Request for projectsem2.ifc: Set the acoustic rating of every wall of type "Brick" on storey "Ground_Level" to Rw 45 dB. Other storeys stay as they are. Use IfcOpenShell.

First a look at what the model holds.

```python
import ifcopenshell
import ifcopenshell.util.element

model = ifcopenshell.open("projectsem2.ifc")
print(model.schema)
storey = next(s for s in model.by_type("IfcBuildingStorey") if s.Name == "Ground_Level")
walls = [e for e in ifcopenshell.util.element.get_decomposition(storey) if e.is_a("IfcWall")]
seen = {}
for e in walls:
    element_type = ifcopenshell.util.element.get_type(e)
    key = (element_type.Name if element_type != e and element_type else None, ifcopenshell.util.element.get_pset(e, "Pset_WallCommon", "AcousticRating"))
    seen[key] = seen.get(key, 0) + 1
for (name, value), count in sorted(seen.items(), key=str):
    print(count, "x", name, "|", value)
```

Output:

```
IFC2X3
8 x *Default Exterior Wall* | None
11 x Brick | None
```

```python
import ifcopenshell
import ifcopenshell.api.pset
import ifcopenshell.util.element

model = ifcopenshell.open("projectsem2.ifc")

storey = next(s for s in model.by_type("IfcBuildingStorey") if s.Name == "Ground_Level")
walls = [e for e in ifcopenshell.util.element.get_decomposition(storey) if e.is_a("IfcWall")]

count = 0
for e in walls:
    element_type = ifcopenshell.util.element.get_type(e)
    if element_type in (None, e) or element_type.Name != "Brick":
        continue
    # add_pset returns the element's existing set when there is one.
    pset = ifcopenshell.api.pset.add_pset(model, product=e, name="Pset_WallCommon")
    ifcopenshell.api.pset.edit_pset(model, pset=pset, properties={"AcousticRating": "Rw 45 dB"})
    count += 1

print(count, "walls updated")

model.write("projectsem2_rev.ifc")
```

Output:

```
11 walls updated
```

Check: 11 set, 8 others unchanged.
